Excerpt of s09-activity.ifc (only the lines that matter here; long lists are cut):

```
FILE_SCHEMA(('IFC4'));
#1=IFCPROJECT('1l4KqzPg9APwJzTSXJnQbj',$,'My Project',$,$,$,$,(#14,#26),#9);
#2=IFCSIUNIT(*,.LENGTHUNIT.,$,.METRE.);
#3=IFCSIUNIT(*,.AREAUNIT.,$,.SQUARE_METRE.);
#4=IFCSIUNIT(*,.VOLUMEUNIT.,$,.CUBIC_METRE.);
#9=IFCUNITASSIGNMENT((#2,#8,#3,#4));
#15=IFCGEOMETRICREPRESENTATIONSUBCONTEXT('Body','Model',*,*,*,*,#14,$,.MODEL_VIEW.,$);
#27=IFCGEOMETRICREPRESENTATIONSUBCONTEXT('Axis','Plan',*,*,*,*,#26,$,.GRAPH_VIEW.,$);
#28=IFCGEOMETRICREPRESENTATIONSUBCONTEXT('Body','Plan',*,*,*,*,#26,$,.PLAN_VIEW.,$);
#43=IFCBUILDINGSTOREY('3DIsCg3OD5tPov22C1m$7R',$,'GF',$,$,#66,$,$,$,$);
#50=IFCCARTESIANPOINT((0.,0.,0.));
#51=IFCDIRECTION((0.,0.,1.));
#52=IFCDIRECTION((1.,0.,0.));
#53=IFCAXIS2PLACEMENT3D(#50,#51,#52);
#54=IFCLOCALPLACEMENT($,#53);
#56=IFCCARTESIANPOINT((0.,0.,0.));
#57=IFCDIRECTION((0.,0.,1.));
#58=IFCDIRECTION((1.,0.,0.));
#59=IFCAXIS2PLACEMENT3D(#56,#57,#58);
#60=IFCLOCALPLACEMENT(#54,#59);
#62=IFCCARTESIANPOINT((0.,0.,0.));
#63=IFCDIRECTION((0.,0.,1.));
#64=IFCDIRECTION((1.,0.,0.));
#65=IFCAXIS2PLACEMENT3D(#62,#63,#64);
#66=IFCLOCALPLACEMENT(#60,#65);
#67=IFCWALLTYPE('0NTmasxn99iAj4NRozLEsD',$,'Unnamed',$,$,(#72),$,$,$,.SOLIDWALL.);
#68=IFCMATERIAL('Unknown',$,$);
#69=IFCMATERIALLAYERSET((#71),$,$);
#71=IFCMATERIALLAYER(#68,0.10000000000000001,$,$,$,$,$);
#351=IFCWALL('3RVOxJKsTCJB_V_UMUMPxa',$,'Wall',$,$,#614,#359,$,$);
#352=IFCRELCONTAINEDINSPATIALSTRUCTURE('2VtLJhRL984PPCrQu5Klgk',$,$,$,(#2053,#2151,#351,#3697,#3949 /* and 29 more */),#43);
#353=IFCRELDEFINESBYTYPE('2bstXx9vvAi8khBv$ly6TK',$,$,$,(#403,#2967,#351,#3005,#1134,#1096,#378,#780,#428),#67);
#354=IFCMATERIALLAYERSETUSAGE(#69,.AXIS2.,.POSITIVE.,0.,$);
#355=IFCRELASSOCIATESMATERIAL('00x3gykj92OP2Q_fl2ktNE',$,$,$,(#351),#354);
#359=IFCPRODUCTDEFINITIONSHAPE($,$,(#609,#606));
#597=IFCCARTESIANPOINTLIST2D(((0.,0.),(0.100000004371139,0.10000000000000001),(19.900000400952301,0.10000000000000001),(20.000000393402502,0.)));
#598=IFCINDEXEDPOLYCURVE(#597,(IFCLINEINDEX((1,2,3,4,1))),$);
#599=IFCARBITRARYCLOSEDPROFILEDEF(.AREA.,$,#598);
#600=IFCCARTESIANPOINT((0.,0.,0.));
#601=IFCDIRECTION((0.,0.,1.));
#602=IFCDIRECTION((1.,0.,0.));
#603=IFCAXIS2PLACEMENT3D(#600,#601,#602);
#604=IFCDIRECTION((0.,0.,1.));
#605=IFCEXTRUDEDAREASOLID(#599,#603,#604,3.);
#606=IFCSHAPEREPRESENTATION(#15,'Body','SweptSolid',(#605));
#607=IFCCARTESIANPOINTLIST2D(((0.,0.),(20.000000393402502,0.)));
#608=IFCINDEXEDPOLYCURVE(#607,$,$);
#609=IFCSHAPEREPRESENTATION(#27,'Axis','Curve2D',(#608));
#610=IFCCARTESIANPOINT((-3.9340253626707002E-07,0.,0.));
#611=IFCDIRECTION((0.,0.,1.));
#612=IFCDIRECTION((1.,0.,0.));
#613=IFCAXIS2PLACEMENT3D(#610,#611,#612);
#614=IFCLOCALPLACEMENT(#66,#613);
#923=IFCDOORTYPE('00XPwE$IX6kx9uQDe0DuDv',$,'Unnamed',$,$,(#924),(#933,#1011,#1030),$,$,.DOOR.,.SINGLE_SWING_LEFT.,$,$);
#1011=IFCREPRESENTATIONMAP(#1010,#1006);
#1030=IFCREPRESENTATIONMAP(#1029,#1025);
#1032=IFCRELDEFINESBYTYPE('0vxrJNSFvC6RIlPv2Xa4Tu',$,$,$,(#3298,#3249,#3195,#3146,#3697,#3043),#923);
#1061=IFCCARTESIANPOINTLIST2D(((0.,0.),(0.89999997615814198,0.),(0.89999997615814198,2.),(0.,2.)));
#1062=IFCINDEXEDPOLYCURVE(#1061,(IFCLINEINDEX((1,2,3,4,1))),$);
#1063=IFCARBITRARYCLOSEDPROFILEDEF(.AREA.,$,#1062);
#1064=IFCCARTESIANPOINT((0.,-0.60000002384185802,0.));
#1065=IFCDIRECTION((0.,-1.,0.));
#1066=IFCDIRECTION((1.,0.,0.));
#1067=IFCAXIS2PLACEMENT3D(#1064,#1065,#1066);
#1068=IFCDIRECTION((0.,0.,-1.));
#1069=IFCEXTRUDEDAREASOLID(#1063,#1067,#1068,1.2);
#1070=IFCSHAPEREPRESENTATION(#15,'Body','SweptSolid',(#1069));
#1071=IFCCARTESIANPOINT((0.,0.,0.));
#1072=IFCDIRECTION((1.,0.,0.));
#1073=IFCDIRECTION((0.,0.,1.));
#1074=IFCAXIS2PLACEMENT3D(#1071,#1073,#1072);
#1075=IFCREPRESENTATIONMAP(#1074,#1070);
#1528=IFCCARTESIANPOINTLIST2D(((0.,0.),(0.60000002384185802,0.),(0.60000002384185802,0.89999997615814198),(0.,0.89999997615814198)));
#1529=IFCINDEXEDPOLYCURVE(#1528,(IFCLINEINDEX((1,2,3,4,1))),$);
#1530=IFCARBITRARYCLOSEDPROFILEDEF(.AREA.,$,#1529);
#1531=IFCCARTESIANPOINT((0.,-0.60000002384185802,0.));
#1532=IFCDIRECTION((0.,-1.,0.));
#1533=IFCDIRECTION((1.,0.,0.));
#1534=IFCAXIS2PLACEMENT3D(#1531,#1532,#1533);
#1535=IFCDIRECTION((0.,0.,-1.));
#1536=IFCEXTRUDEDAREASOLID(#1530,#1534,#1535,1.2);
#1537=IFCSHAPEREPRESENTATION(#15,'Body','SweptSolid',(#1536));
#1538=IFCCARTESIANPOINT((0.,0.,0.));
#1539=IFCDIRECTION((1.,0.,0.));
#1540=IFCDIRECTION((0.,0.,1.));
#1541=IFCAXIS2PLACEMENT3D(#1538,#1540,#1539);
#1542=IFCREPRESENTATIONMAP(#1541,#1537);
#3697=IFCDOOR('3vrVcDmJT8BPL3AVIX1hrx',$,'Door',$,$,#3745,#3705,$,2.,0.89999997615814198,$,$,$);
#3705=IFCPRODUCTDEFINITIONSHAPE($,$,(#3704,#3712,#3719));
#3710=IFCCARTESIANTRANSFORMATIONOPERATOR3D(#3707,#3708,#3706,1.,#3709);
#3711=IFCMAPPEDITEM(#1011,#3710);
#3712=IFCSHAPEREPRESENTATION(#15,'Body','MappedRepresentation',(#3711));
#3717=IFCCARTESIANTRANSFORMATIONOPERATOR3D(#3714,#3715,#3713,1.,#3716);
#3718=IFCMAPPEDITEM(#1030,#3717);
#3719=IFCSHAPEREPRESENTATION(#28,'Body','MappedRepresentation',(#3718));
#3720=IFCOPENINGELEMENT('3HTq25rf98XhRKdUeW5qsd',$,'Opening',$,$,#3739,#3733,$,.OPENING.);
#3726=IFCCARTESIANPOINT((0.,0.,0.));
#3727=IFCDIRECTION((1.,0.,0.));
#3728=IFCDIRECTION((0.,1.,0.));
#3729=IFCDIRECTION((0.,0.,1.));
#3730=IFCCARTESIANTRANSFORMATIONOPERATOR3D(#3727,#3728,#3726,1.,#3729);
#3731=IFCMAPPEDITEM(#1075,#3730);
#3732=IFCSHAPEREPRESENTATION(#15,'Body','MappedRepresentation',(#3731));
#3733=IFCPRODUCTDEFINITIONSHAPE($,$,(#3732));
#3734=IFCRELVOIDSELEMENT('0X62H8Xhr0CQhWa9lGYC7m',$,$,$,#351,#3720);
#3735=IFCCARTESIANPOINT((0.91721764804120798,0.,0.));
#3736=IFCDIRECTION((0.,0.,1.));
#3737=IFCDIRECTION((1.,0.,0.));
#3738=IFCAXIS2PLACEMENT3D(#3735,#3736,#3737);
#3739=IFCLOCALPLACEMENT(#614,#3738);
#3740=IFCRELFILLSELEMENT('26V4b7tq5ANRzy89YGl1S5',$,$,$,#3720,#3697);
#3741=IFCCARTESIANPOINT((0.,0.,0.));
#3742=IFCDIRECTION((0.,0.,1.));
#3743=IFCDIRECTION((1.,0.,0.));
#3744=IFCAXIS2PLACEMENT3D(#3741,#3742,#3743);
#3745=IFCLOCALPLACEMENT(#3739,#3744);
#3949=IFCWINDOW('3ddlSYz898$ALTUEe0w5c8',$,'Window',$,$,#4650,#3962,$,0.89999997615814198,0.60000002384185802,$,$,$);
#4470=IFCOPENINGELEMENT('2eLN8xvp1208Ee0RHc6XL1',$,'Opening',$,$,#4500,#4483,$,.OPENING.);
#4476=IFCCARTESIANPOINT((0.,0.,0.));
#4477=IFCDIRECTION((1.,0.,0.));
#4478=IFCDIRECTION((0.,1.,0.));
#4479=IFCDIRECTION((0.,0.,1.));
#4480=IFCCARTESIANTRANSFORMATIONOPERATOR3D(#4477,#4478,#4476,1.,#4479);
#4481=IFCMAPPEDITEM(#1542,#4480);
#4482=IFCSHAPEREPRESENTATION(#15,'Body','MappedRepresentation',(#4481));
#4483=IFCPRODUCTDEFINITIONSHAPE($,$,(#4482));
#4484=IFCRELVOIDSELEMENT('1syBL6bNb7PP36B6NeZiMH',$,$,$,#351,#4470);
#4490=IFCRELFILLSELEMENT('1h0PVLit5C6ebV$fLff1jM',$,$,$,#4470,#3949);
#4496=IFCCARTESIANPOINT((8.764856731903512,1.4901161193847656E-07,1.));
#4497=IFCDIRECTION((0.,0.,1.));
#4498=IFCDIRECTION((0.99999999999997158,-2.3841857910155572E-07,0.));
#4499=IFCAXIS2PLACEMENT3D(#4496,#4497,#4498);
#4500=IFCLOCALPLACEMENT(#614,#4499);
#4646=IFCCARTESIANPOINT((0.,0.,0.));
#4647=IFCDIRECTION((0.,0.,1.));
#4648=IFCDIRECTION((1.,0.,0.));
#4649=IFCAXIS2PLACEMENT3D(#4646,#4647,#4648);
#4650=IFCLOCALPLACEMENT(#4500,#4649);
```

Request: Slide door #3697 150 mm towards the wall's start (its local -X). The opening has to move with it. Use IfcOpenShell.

```python
import ifcopenshell
import ifcopenshell.api.geometry
import ifcopenshell.util.placement

model = ifcopenshell.open("s09-activity.ifc")

door = model.by_guid("3vrVcDmJT8BPL3AVIX1hrx")
opening = door.FillsVoids[0].RelatingOpeningElement
wall = opening.VoidsElements[0].RelatingBuildingElement

wall_matrix = ifcopenshell.util.placement.get_local_placement(wall.ObjectPlacement)
shift = wall_matrix[:3, 0] * -0.15
before = ifcopenshell.util.placement.get_local_placement(door.ObjectPlacement)[:3, 3].copy()

# The door is placed relative to its opening, so it follows when the opening moves.
matrix = ifcopenshell.util.placement.get_local_placement(opening.ObjectPlacement)
matrix[:3, 3] += shift
ifcopenshell.api.geometry.edit_object_placement(
    model, product=opening, matrix=matrix, is_si=False, should_transform_children=True
)

after = ifcopenshell.util.placement.get_local_placement(door.ObjectPlacement)[:3, 3]
print("door moved by", (after - before).round(3) + 0.0)

model.write("s09-activity_v2.ifc")
```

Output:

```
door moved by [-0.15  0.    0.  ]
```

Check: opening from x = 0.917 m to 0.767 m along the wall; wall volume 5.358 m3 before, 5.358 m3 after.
